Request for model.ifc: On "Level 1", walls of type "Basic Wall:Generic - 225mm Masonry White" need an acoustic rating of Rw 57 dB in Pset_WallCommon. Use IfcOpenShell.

First a look at what the model holds.

```python
import ifcopenshell
import ifcopenshell.util.element

model = ifcopenshell.open("model.ifc")
print(model.schema)
storey = next(s for s in model.by_type("IfcBuildingStorey") if s.Name == "Level 1")
walls = [e for e in ifcopenshell.util.element.get_decomposition(storey) if e.is_a("IfcWall")]
seen = {}
for e in walls:
    element_type = ifcopenshell.util.element.get_type(e)
    key = (element_type.Name if element_type != e and element_type else None, ifcopenshell.util.element.get_pset(e, "Pset_WallCommon", "AcousticRating"))
    seen[key] = seen.get(key, 0) + 1
for (name, value), count in sorted(seen.items(), key=str):
    print(count, "x", name, "|", value)
```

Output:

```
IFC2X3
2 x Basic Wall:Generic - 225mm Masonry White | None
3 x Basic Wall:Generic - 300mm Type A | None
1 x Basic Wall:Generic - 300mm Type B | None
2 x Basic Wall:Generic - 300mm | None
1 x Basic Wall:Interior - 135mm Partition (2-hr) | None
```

```python
import ifcopenshell
import ifcopenshell.api.pset
import ifcopenshell.util.element

model = ifcopenshell.open("model.ifc")

storey = next(s for s in model.by_type("IfcBuildingStorey") if s.Name == "Level 1")
walls = [e for e in ifcopenshell.util.element.get_decomposition(storey) if e.is_a("IfcWall")]

count = 0
for e in walls:
    element_type = ifcopenshell.util.element.get_type(e)
    if element_type in (None, e) or element_type.Name != "Basic Wall:Generic - 225mm Masonry White":
        continue
    # add_pset returns the element's existing set when there is one.
    pset = ifcopenshell.api.pset.add_pset(model, product=e, name="Pset_WallCommon")
    ifcopenshell.api.pset.edit_pset(model, pset=pset, properties={"AcousticRating": "Rw 57 dB"})
    count += 1

print(count, "walls updated")

model.write("model_v2.ifc")
```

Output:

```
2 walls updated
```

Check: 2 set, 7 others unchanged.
